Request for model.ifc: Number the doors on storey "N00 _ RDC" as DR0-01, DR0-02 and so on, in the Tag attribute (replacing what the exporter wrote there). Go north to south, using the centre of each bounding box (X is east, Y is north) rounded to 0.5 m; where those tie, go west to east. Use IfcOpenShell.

First a look at what the model holds.

```python
import ifcopenshell
import ifcopenshell.util.element
import ifcopenshell.util.placement

model = ifcopenshell.open("model.ifc")
print(model.schema)
storey = next(s for s in model.by_type("IfcBuildingStorey") if s.Name == "N00 _ RDC")
doors = [e for e in ifcopenshell.util.element.get_decomposition(storey) if e.is_a("IfcDoor")]
for e in sorted(doors, key=lambda e: e.id()):
    origin = ifcopenshell.util.placement.get_local_placement(e.ObjectPlacement)[:3, 3]
    print(e.id(), e.Tag, e.Name, origin.round(2) + 0.0, sep=" | ")
```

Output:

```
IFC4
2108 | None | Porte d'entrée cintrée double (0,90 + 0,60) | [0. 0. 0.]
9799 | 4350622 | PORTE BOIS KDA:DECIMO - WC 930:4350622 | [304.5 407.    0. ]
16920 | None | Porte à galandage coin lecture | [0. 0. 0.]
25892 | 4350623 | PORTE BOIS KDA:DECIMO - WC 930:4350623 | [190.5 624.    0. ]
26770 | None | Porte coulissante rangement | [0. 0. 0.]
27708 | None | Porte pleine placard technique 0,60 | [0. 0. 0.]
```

```python
import ifcopenshell
import ifcopenshell.geom
import ifcopenshell.util.element
import ifcopenshell.util.shape

model = ifcopenshell.open("model.ifc")
settings = ifcopenshell.geom.settings()
settings.set("use-world-coords", True)


def centre(element):
    shape = ifcopenshell.geom.create_shape(settings, element)
    return ifcopenshell.util.shape.get_bbox_centroid(shape.geometry)


storey = next(s for s in model.by_type("IfcBuildingStorey") if s.Name == "N00 _ RDC")
doors = [e for e in ifcopenshell.util.element.get_decomposition(storey) if e.is_a("IfcDoor")]

# Insertion points can sit at a corner or the storey origin, so sort by the geometry (in metres).
centres = {e: centre(e) for e in doors}
doors.sort(key=lambda e: (-round(centres[e][1] / 0.5), centres[e][0]))

for i, e in enumerate(doors, start=1):
    number = f"DR0-{i:02d}"
    e.Tag = number
    print(e.id(), number)

model.write("model_v2.ifc")
```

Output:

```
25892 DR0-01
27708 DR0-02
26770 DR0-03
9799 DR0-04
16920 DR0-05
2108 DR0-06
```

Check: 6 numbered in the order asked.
